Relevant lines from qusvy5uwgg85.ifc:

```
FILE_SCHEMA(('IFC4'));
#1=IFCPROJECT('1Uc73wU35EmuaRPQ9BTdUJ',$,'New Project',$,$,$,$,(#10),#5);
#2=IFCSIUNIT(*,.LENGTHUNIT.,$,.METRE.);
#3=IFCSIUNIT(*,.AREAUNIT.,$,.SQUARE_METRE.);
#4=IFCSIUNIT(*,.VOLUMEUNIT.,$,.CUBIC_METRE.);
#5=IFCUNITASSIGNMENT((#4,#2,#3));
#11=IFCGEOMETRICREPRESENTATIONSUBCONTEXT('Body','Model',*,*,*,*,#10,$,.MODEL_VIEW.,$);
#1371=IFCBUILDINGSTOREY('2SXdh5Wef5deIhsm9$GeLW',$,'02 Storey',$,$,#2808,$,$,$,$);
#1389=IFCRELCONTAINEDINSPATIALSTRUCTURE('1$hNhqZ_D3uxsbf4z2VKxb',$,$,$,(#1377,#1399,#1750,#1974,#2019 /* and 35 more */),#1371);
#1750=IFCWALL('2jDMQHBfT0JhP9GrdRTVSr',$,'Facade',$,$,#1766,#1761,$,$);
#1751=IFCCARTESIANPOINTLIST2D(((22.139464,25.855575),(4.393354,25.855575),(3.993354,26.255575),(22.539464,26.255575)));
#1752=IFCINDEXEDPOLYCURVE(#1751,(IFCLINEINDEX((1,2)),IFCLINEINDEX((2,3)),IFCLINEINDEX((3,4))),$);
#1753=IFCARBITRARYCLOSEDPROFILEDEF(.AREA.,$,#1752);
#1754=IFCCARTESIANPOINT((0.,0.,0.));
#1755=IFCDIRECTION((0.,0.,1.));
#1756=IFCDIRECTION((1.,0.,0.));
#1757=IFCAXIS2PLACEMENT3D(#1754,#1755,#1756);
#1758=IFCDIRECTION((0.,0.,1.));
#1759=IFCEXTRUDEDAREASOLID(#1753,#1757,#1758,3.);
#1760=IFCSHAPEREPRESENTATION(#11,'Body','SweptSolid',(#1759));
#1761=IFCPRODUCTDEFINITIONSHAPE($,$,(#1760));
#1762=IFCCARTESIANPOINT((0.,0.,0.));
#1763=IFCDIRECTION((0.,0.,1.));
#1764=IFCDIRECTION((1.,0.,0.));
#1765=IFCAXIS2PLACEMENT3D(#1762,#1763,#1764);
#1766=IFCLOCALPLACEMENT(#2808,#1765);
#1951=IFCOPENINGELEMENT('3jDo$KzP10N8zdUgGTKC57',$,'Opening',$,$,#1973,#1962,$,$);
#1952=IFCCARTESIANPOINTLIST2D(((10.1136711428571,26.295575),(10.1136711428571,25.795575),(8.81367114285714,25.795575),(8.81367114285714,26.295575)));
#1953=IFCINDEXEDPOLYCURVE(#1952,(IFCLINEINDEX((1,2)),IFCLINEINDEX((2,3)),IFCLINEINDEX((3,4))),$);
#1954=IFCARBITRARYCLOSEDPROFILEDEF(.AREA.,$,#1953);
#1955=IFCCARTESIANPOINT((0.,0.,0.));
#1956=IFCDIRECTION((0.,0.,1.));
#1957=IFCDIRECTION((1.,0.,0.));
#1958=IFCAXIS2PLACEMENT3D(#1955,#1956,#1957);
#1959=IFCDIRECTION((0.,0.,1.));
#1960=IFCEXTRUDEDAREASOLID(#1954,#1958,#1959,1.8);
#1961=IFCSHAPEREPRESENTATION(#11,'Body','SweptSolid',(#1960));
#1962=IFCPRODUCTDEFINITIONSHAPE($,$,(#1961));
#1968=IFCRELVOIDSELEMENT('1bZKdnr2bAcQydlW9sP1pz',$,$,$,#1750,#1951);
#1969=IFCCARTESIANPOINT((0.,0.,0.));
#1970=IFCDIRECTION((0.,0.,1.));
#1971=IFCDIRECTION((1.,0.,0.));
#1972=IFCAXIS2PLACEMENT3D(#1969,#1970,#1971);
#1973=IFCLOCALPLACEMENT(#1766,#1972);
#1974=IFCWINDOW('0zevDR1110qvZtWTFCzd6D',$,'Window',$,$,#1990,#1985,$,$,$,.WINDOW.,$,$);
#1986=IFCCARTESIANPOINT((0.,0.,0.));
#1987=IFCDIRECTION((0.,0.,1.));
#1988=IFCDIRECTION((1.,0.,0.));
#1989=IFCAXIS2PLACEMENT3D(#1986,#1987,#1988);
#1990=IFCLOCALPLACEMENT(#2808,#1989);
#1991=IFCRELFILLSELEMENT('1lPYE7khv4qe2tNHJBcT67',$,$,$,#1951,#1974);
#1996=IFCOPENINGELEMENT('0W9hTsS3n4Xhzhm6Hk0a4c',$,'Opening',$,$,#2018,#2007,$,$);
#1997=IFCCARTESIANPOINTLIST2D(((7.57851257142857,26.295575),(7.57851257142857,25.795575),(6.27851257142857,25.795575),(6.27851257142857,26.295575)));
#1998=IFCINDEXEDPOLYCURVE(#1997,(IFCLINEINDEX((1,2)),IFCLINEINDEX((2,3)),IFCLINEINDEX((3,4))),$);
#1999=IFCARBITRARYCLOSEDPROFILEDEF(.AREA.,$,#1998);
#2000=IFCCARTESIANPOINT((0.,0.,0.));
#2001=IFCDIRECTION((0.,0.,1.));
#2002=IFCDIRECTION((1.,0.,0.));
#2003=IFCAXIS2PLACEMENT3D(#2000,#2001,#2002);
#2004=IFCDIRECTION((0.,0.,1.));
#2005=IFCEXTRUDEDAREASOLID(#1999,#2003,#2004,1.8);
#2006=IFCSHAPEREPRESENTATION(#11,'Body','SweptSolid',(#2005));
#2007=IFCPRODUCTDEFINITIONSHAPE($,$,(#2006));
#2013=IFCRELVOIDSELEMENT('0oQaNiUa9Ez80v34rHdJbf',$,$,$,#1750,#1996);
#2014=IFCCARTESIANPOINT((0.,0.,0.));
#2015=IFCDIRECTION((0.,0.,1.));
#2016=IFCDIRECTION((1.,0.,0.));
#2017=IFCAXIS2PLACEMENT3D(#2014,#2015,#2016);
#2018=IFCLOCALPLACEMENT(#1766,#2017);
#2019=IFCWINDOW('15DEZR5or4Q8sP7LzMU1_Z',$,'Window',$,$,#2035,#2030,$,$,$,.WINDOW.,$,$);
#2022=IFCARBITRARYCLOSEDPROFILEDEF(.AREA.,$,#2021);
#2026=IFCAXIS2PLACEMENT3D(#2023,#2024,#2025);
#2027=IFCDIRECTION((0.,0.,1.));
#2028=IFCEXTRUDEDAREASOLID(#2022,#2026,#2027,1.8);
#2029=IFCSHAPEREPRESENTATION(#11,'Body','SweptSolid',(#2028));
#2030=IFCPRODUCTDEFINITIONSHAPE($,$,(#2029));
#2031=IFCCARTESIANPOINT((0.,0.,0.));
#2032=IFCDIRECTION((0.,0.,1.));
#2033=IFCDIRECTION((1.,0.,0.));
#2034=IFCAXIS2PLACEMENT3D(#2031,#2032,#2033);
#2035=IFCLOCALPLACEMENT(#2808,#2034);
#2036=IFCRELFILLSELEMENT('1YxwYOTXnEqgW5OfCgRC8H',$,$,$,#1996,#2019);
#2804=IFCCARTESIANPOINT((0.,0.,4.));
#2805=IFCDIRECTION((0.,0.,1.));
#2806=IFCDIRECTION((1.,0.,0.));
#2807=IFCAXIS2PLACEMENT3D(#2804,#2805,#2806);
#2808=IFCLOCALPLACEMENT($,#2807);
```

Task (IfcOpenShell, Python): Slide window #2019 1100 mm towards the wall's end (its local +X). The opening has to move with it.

```python
import ifcopenshell
import ifcopenshell.api.geometry
import ifcopenshell.util.placement

model = ifcopenshell.open("qusvy5uwgg85.ifc")

window = model.by_guid("15DEZR5or4Q8sP7LzMU1_Z")
opening = window.FillsVoids[0].RelatingOpeningElement
wall = opening.VoidsElements[0].RelatingBuildingElement

wall_matrix = ifcopenshell.util.placement.get_local_placement(wall.ObjectPlacement)
shift = wall_matrix[:3, 0] * 1.1
before = ifcopenshell.util.placement.get_local_placement(window.ObjectPlacement)[:3, 3].copy()

# The window is not placed relative to its opening, so move both.
for product in (opening, window):
    matrix = ifcopenshell.util.placement.get_local_placement(product.ObjectPlacement)
    matrix[:3, 3] += shift
    ifcopenshell.api.geometry.edit_object_placement(model, product=product, matrix=matrix, is_si=False)

after = ifcopenshell.util.placement.get_local_placement(window.ObjectPlacement)[:3, 3]
print("window moved by", (after - before).round(3) + 0.0)

model.write("qusvy5uwgg85_edited.ifc")
```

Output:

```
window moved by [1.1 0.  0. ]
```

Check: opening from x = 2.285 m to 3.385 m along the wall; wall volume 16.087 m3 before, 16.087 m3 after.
